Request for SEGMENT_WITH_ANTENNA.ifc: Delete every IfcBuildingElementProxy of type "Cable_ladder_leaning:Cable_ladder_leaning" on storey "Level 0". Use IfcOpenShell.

First a look at what the model holds.

```python
import ifcopenshell
import ifcopenshell.util.element

model = ifcopenshell.open("SEGMENT_WITH_ANTENNA.ifc")
print(model.schema)
storey = next(s for s in model.by_type("IfcBuildingStorey") if s.Name == "Level 0")
proxies = [e for e in ifcopenshell.util.element.get_decomposition(storey) if e.is_a("IfcBuildingElementProxy")]
seen = {}
for e in proxies:
    element_type = ifcopenshell.util.element.get_type(e)
    name = element_type.Name if element_type not in (None, e) else None
    seen[name] = seen.get(name, 0) + 1
for name, count in sorted(seen.items(), key=str):
    print(count, "x", name)
```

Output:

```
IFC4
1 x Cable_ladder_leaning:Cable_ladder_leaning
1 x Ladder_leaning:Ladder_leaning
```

```python
import ifcopenshell
import ifcopenshell.api.root
import ifcopenshell.util.element

model = ifcopenshell.open("SEGMENT_WITH_ANTENNA.ifc")

storey = next(s for s in model.by_type("IfcBuildingStorey") if s.Name == "Level 0")
proxies = [e for e in ifcopenshell.util.element.get_decomposition(storey) if e.is_a("IfcBuildingElementProxy")]
targets = [e for e in proxies if (t := ifcopenshell.util.element.get_type(e)) not in (None, e) and t.Name == "Cable_ladder_leaning:Cable_ladder_leaning"]

for e in targets:
    ifcopenshell.api.root.remove_product(model, product=e)
print(len(targets), "removed")

model.write("SEGMENT_WITH_ANTENNA_edited.ifc")
```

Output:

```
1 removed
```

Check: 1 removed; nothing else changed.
